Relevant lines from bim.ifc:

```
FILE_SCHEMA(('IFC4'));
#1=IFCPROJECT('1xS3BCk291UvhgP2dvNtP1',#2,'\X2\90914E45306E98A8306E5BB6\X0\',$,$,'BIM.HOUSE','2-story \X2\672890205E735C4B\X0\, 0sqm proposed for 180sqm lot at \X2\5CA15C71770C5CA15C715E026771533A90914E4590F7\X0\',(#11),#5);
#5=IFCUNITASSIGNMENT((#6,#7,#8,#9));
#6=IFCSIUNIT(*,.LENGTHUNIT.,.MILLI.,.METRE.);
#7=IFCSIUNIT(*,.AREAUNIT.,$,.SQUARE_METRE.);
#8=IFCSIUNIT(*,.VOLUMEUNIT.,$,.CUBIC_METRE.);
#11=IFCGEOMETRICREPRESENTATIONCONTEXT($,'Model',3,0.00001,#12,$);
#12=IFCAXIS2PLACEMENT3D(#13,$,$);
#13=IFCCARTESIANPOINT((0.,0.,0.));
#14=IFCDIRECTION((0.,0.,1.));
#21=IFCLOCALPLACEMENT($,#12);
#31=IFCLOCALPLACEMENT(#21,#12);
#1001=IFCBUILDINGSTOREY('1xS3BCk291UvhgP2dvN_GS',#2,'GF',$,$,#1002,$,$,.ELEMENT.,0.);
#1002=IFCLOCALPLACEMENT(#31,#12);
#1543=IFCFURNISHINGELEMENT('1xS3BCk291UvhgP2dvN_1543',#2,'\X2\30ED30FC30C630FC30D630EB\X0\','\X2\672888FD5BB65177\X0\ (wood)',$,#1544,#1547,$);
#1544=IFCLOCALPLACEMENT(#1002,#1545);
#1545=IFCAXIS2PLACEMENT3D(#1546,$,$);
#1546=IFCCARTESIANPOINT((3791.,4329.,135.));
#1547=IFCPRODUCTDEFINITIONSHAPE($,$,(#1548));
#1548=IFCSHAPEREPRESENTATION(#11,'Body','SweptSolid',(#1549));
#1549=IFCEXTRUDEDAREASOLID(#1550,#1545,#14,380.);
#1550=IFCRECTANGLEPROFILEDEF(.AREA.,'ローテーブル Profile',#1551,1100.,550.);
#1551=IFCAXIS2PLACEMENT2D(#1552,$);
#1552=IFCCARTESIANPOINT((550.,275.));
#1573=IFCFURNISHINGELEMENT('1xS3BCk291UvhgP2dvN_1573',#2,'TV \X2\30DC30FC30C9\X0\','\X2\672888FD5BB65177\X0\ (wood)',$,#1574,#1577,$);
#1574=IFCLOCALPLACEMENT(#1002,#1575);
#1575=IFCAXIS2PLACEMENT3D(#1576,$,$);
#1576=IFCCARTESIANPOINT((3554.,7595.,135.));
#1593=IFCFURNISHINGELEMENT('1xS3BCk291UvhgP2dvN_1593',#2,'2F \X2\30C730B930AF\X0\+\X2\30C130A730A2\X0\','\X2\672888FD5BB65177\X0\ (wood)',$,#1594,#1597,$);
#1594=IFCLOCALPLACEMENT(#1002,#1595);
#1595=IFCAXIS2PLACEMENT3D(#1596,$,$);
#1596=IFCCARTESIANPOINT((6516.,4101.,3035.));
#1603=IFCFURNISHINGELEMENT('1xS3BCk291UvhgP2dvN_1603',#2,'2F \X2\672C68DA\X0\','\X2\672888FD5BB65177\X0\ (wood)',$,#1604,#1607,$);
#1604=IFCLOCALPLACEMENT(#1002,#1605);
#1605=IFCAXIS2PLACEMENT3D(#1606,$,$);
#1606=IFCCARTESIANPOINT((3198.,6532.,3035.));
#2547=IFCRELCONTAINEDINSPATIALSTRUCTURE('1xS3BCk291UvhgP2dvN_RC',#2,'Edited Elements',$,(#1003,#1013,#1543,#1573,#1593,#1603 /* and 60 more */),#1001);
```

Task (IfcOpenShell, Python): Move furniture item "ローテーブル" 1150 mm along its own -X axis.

```python
import ifcopenshell
import ifcopenshell.api.geometry
import ifcopenshell.util.placement
import ifcopenshell.util.unit

model = ifcopenshell.open("bim.ifc")
unit_scale = ifcopenshell.util.unit.calculate_unit_scale(model)

item = model.by_id(1543)
matrix = ifcopenshell.util.placement.get_local_placement(item.ObjectPlacement)
matrix[:3, 3] -= matrix[:3, 0] * 1.15 / unit_scale
ifcopenshell.api.geometry.edit_object_placement(model, product=item, matrix=matrix, is_si=False)

print(ifcopenshell.util.placement.get_local_placement(item.ObjectPlacement).round(3) + 0.0)

model.write("bim_updated.ifc")
```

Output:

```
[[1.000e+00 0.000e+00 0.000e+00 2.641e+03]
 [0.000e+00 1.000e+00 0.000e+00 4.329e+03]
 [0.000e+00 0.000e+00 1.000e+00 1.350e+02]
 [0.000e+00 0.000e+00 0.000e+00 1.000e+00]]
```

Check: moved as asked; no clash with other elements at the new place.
